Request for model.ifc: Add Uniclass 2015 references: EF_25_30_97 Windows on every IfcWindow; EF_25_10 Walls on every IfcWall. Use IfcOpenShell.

First a look at what the model holds.

```python
import ifcopenshell

model = ifcopenshell.open("model.ifc")
print(model.schema)
print("classifications:", [c.Name for c in model.by_type("IfcClassification")])
for ifc_class in ("IfcDoor", "IfcRoof", "IfcStair", "IfcWall", "IfcWindow"):
    print(ifc_class, len(model.by_type(ifc_class)))
```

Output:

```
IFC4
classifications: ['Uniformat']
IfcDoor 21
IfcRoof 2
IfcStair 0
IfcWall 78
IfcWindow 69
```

```python
import ifcopenshell
import ifcopenshell.api.classification

model = ifcopenshell.open("model.ifc")

system = ifcopenshell.api.classification.add_classification(model, classification="Uniclass 2015")

codes = {
    "IfcWindow": ("EF_25_30_97", "Windows"),
    "IfcWall": ("EF_25_10", "Walls"),
}
for ifc_class, (code, name) in codes.items():
    products = model.by_type(ifc_class)
    ifcopenshell.api.classification.add_reference(
        model, products=products, classification=system, identification=code, name=name
    )
    print(code, len(products))

model.write("model_rev.ifc")
```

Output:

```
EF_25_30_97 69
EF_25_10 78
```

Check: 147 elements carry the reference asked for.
